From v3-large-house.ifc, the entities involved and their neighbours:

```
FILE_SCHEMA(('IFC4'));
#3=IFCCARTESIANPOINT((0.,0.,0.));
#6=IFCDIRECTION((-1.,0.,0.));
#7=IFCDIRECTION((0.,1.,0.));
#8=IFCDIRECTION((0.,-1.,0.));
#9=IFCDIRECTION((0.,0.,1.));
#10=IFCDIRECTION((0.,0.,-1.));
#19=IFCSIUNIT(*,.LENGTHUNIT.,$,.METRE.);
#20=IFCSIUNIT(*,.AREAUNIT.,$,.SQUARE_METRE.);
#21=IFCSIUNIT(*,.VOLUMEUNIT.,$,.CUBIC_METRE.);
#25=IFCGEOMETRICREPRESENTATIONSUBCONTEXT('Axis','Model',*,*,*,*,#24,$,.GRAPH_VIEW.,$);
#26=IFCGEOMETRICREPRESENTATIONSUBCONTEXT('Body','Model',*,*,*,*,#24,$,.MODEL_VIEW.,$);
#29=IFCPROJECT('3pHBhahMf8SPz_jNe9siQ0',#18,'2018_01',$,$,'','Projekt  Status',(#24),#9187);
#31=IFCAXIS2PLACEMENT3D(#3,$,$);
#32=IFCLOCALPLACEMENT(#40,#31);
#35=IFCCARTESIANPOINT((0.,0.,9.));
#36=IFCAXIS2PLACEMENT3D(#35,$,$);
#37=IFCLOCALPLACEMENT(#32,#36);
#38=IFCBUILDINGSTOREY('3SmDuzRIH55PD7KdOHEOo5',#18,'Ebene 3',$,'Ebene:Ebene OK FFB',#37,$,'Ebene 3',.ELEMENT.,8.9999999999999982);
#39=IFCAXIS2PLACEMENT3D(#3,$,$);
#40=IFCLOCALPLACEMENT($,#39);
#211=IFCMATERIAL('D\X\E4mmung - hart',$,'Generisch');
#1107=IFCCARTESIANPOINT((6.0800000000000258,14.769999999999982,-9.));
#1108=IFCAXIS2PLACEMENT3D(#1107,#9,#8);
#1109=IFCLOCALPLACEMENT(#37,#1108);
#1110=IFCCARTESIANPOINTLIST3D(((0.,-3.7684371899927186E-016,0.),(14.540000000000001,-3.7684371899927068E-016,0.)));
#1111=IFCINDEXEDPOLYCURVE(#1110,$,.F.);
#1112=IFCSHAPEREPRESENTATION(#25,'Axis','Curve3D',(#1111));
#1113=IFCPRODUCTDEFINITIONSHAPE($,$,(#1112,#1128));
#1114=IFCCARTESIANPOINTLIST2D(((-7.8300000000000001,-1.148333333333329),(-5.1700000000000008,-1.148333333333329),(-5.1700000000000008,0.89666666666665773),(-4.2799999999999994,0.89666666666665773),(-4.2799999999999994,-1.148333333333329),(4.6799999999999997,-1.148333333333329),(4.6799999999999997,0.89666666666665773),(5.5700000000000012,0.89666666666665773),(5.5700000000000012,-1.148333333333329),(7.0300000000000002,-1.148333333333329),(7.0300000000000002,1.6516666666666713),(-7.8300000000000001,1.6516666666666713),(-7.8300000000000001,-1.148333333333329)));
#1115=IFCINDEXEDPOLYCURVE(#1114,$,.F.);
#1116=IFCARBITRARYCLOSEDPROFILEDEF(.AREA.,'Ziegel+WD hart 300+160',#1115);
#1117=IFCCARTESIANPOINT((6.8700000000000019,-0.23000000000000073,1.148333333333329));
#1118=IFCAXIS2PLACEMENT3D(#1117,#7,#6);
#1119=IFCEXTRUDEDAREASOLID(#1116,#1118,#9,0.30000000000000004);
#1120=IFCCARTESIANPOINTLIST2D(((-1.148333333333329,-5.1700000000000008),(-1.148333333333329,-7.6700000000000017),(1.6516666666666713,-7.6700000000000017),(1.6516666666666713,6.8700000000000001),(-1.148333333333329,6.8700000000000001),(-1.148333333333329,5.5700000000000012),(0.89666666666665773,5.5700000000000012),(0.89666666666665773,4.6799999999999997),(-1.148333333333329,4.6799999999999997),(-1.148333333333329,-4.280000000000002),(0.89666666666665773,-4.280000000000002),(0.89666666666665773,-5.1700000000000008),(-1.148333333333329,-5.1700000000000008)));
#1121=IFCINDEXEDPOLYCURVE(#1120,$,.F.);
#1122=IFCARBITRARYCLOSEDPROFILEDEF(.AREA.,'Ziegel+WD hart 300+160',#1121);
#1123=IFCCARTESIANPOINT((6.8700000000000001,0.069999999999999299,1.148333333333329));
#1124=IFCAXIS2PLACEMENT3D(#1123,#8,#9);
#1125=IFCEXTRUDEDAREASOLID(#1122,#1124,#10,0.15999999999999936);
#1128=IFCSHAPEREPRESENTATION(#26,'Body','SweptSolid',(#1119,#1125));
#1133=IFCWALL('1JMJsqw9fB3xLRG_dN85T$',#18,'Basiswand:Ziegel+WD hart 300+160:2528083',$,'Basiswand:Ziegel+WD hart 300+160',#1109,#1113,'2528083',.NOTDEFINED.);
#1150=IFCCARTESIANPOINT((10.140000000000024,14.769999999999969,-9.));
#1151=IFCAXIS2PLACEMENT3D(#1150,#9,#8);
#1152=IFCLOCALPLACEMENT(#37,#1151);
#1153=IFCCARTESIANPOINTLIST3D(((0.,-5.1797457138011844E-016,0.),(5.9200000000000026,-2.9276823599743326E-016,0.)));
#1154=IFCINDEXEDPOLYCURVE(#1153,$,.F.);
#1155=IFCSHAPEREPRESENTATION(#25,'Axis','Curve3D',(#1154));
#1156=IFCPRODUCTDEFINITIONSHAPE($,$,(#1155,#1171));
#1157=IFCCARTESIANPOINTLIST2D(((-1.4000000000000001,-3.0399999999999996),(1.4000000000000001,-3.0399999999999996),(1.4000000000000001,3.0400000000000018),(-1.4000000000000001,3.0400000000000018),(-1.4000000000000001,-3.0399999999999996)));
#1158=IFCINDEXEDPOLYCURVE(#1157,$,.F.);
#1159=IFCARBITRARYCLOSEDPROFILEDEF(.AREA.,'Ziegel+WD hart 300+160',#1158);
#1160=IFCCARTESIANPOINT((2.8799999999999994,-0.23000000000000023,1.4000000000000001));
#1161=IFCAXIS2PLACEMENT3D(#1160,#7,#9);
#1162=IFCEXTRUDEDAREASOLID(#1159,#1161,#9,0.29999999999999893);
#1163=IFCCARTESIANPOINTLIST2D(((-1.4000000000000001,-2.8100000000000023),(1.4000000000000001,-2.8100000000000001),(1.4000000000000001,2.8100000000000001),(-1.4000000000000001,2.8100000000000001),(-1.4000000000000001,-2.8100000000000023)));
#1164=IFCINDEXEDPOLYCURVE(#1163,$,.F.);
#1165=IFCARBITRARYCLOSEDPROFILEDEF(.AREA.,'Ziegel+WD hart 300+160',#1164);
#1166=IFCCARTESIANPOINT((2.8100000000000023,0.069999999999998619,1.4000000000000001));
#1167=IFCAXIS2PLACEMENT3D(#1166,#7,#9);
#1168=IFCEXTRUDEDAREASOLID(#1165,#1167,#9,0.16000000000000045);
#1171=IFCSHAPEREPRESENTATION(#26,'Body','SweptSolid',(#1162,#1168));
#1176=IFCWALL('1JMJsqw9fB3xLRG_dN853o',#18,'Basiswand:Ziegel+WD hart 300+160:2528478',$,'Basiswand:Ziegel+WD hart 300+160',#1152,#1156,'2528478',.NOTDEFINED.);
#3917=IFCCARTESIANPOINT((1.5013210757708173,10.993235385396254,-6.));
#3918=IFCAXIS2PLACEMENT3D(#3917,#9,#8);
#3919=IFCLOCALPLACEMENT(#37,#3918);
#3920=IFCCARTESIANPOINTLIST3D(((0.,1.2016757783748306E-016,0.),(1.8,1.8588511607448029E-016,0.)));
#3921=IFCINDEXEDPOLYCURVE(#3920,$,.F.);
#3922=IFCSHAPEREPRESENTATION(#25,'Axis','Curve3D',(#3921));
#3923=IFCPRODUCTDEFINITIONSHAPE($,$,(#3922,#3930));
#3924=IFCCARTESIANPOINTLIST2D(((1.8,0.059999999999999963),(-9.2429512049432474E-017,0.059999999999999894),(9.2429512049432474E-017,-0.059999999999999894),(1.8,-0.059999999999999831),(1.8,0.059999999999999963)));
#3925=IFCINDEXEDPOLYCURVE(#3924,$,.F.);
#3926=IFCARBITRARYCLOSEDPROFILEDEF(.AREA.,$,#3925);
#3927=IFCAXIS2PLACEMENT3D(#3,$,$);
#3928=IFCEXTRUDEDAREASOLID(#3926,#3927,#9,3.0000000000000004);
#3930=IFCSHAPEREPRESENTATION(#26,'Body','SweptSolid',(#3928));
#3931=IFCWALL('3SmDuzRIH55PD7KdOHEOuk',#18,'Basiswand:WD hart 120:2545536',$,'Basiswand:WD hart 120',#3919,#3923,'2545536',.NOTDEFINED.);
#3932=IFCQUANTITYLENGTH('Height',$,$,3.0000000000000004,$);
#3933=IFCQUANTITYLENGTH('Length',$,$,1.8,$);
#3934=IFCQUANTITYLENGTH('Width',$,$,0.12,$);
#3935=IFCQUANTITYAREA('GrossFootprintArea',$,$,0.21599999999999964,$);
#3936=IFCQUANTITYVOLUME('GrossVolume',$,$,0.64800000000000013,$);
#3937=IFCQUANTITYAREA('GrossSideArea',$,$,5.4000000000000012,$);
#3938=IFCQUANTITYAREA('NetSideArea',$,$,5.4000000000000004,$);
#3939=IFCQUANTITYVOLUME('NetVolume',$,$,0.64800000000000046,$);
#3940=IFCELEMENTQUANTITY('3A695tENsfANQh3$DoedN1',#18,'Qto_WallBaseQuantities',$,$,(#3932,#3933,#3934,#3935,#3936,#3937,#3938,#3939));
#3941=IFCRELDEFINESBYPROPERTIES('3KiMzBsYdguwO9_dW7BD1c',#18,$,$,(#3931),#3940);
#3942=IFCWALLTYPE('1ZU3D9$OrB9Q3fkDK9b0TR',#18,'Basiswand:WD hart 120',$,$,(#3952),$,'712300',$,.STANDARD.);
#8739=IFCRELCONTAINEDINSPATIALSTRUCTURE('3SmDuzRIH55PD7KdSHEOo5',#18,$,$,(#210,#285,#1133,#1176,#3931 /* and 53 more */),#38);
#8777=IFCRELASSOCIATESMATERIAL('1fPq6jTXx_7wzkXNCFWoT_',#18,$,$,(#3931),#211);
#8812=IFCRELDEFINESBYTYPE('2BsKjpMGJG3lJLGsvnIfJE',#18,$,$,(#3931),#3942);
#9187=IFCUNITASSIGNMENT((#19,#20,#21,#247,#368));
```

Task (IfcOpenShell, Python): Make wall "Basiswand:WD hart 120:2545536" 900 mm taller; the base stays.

```python
import ifcopenshell
import ifcopenshell.api.pset
import ifcopenshell.geom
import ifcopenshell.util.element
import ifcopenshell.util.representation
import ifcopenshell.util.shape
import ifcopenshell.util.unit

model = ifcopenshell.open("v3-large-house.ifc")
unit_scale = ifcopenshell.util.unit.calculate_unit_scale(model)
area_scale = ifcopenshell.util.unit.calculate_unit_scale(model, "AREAUNIT")
volume_scale = ifcopenshell.util.unit.calculate_unit_scale(model, "VOLUMEUNIT")
settings = ifcopenshell.geom.settings()


def volume(element):
    """Net volume in cubic metres, openings subtracted."""
    shape = ifcopenshell.geom.create_shape(settings, element)
    return ifcopenshell.util.shape.get_volume(shape.geometry)


wall = model.by_id(3931)
before = volume(wall)

body = ifcopenshell.util.representation.get_representation(wall, "Model", "Body")
solid = body.Items[0]
old_height = solid.Depth
solid.Depth += 0.9 / unit_scale
after = volume(wall)
thickness = 0.12  # wall thickness in metres

# Update the stored height, areas and volumes.
qto = model.by_id(ifcopenshell.util.element.get_pset(wall, "Qto_WallBaseQuantities", should_inherit=False)["id"])
ifcopenshell.api.pset.edit_qto(model, qto=qto, properties={
    "Height": solid.Depth,
    "GrossVolume": ifcopenshell.util.element.get_pset(wall, "Qto_WallBaseQuantities", "GrossVolume") * solid.Depth / old_height,
    "GrossSideArea": ifcopenshell.util.element.get_pset(wall, "Qto_WallBaseQuantities", "GrossSideArea") * solid.Depth / old_height,
    "NetSideArea": after / thickness / area_scale,
    "NetVolume": after / volume_scale,
})

print(f"height {old_height:g} -> {solid.Depth:g}, volume {before:.3f} -> {after:.3f} m3")

model.write("v3-large-house_rev.ifc")
```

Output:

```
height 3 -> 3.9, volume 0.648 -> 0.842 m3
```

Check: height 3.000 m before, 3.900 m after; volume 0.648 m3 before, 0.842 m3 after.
